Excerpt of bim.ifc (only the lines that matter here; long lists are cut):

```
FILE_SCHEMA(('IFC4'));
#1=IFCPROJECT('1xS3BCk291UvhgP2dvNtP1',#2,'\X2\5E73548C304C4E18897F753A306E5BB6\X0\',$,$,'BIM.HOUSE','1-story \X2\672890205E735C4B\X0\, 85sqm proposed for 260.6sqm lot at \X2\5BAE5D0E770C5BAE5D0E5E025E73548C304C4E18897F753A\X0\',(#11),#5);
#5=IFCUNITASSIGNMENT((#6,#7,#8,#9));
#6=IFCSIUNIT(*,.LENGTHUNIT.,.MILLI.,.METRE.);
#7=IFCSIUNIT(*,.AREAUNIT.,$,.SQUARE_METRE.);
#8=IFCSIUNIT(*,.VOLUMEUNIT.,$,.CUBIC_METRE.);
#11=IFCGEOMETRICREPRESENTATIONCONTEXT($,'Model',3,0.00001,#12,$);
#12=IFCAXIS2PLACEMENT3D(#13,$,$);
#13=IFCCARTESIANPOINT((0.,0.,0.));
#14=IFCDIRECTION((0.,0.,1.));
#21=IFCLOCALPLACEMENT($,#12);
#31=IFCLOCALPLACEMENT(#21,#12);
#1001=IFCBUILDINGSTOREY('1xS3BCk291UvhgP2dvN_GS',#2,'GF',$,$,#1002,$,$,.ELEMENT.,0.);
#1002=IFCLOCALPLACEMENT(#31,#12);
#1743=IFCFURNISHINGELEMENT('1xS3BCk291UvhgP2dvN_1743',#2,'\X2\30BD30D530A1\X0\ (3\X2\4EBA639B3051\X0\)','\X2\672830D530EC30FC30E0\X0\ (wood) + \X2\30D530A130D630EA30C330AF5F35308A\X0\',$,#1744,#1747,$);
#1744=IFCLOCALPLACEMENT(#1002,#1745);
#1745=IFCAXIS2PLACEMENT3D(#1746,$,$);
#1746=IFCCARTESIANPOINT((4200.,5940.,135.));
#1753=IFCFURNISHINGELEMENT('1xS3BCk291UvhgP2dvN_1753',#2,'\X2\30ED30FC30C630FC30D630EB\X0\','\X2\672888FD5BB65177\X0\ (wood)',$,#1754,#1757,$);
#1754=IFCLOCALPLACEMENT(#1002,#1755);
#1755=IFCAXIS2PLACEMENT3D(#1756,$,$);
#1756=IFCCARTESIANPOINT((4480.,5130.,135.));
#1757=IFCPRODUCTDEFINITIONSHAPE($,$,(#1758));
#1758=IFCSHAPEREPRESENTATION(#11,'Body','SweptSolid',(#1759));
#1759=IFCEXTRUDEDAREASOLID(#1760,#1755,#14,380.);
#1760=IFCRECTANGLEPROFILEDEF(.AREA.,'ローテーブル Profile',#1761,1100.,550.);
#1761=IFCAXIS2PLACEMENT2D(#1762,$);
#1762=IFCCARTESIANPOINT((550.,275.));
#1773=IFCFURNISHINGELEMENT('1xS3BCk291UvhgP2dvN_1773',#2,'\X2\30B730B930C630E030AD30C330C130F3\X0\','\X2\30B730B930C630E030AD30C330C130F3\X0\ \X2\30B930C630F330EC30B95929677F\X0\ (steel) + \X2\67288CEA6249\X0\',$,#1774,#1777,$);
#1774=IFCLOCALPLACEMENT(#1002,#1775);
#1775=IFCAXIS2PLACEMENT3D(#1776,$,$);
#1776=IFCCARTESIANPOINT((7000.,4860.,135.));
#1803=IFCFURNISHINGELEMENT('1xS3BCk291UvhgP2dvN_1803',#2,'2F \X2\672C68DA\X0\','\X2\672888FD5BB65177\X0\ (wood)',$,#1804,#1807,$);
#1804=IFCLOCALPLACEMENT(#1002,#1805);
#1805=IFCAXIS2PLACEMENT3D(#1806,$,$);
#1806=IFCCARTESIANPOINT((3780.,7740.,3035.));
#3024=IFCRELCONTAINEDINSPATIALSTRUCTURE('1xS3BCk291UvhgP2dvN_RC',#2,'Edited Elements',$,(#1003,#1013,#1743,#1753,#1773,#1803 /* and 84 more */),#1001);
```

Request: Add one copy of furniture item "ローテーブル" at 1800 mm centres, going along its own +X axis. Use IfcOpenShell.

```python
import ifcopenshell
import ifcopenshell.api.geometry
import ifcopenshell.api.root
import ifcopenshell.util.element
import ifcopenshell.util.placement
import ifcopenshell.util.unit

model = ifcopenshell.open("bim.ifc")
unit_scale = ifcopenshell.util.unit.calculate_unit_scale(model)


def reuse_history(source, copy):
    """copy_class also copies each property set's owner history, people and application; keep the originals."""
    for rel in copy.IsDefinedBy:
        if rel.is_a("IfcRelDefinesByProperties") and (history := rel.RelatingPropertyDefinition.OwnerHistory):
            rel.RelatingPropertyDefinition.OwnerHistory = source.OwnerHistory
            ifcopenshell.util.element.remove_deep2(model, history)


source = model.by_id(1753)
base = ifcopenshell.util.placement.get_local_placement(source.ObjectPlacement)
step = base[:3, 0] * 1.8 / unit_scale

for i in range(1, 2):
    copy = ifcopenshell.api.root.copy_class(model, product=source)
    copy.Representation = ifcopenshell.util.element.copy_deep(
        model, source.Representation, exclude=["IfcGeometricRepresentationContext", "IfcRepresentationMap"]
    )
    reuse_history(source, copy)
    matrix = base.copy()
    matrix[:3, 3] += i * step
    print("added at", matrix[:3, 3].round(3) + 0.0)
    ifcopenshell.api.geometry.edit_object_placement(model, product=copy, matrix=matrix, is_si=False)

model.write("bim_updated.ifc")
```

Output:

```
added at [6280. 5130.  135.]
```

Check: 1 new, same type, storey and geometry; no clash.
